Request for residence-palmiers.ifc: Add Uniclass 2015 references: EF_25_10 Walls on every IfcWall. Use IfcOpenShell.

First a look at what the model holds.

```python
import ifcopenshell

model = ifcopenshell.open("residence-palmiers.ifc")
print(model.schema)
print("classifications:", [c.Name for c in model.by_type("IfcClassification")])
for ifc_class in ("IfcDoor", "IfcRoof", "IfcStair", "IfcWall", "IfcWindow"):
    print(ifc_class, len(model.by_type(ifc_class)))
```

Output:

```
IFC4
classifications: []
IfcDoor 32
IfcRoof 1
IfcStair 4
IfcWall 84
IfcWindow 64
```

```python
import ifcopenshell
import ifcopenshell.api.classification

model = ifcopenshell.open("residence-palmiers.ifc")

system = ifcopenshell.api.classification.add_classification(model, classification="Uniclass 2015")

codes = {
    "IfcWall": ("EF_25_10", "Walls"),
}
for ifc_class, (code, name) in codes.items():
    products = model.by_type(ifc_class)
    ifcopenshell.api.classification.add_reference(
        model, products=products, classification=system, identification=code, name=name
    )
    print(code, len(products))

model.write("residence-palmiers-out.ifc")
```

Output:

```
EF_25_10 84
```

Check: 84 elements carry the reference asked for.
